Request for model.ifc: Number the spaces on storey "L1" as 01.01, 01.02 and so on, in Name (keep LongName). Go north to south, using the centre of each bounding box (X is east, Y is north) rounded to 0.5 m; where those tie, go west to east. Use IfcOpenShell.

First a look at what the model holds.

```python
import ifcopenshell
import ifcopenshell.util.element
import ifcopenshell.util.placement

model = ifcopenshell.open("model.ifc")
print(model.schema)
storey = next(s for s in model.by_type("IfcBuildingStorey") if s.Name == "L1")
spaces = [e for e in ifcopenshell.util.element.get_decomposition(storey) if e.is_a("IfcSpace")]
for e in sorted(spaces, key=lambda e: e.id()):
    origin = ifcopenshell.util.placement.get_local_placement(e.ObjectPlacement)[:3, 3]
    print(e.id(), e.Name, e.LongName, origin.round(2) + 0.0, sep=" | ")
```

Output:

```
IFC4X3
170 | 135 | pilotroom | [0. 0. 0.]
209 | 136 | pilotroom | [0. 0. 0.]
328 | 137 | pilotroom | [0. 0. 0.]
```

```python
import ifcopenshell
import ifcopenshell.geom
import ifcopenshell.util.element
import ifcopenshell.util.shape

model = ifcopenshell.open("model.ifc")
settings = ifcopenshell.geom.settings()
settings.set("use-world-coords", True)


def centre(element):
    shape = ifcopenshell.geom.create_shape(settings, element)
    return ifcopenshell.util.shape.get_bbox_centroid(shape.geometry)


storey = next(s for s in model.by_type("IfcBuildingStorey") if s.Name == "L1")
spaces = [e for e in ifcopenshell.util.element.get_decomposition(storey) if e.is_a("IfcSpace")]

# Insertion points can sit at a corner or the storey origin, so sort by the geometry (in metres).
centres = {e: centre(e) for e in spaces}
spaces.sort(key=lambda e: (-round(centres[e][1] / 0.5), centres[e][0]))

for i, e in enumerate(spaces, start=1):
    number = f"01.{i:02d}"
    e.Name = number
    print(e.id(), number)

model.write("model-out.ifc")
```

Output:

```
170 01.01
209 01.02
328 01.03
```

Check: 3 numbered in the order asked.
